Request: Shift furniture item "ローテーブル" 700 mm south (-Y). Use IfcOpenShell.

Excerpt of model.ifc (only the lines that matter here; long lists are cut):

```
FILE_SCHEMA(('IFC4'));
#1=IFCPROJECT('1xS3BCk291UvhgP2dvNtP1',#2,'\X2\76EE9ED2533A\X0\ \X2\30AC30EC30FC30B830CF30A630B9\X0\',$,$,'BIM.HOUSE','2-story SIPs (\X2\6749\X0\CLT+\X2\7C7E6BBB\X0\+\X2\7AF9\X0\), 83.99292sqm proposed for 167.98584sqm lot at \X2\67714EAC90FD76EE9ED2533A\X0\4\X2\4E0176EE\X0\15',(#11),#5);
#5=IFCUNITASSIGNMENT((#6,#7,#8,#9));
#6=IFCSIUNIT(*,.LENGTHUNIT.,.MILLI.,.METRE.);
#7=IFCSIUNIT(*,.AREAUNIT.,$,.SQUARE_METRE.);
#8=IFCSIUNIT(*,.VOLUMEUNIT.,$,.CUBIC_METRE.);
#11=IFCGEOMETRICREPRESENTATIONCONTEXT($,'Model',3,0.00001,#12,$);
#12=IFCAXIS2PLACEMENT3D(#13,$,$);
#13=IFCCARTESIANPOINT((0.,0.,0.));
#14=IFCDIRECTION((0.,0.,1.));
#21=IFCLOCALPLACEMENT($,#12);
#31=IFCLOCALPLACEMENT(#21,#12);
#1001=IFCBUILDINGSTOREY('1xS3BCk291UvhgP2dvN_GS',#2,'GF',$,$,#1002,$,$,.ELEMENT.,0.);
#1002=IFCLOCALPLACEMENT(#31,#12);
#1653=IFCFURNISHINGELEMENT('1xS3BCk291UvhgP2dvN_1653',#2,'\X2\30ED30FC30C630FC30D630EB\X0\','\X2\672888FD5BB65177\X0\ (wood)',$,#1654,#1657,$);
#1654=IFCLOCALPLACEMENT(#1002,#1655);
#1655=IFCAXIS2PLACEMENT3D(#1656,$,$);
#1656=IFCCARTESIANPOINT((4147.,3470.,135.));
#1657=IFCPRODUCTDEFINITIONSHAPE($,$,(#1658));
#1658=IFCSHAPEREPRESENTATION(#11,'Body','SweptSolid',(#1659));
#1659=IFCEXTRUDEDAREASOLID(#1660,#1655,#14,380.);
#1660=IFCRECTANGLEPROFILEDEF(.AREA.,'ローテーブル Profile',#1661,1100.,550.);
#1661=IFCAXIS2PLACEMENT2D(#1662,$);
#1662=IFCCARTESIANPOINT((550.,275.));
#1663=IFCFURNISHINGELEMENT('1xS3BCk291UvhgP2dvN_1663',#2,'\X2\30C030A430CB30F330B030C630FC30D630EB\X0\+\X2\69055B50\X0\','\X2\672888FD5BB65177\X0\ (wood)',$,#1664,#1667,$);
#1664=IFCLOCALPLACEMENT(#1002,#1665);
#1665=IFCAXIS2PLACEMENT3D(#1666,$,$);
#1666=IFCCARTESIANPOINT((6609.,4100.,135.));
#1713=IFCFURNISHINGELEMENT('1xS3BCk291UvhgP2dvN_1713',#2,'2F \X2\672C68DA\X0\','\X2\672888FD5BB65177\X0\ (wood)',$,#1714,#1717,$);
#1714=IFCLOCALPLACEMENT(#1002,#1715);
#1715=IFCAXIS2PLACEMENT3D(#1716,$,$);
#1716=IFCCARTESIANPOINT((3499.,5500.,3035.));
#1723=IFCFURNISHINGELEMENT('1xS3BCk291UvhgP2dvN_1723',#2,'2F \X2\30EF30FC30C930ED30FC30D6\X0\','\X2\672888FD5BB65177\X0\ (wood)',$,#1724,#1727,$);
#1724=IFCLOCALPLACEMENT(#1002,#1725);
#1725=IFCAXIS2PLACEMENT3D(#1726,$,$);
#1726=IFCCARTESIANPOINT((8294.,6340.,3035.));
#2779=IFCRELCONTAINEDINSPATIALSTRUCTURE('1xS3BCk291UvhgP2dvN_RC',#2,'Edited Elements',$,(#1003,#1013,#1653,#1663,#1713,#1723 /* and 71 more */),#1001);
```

```python
import ifcopenshell
import ifcopenshell.api.geometry
import ifcopenshell.util.placement
import ifcopenshell.util.unit

model = ifcopenshell.open("model.ifc")
unit_scale = ifcopenshell.util.unit.calculate_unit_scale(model)

item = model.by_guid("1xS3BCk291UvhgP2dvN_1653")
matrix = ifcopenshell.util.placement.get_local_placement(item.ObjectPlacement)
matrix[1, 3] -= 0.7 / unit_scale
ifcopenshell.api.geometry.edit_object_placement(model, product=item, matrix=matrix, is_si=False)

print(ifcopenshell.util.placement.get_local_placement(item.ObjectPlacement).round(3) + 0.0)

model.write("model_rev.ifc")
```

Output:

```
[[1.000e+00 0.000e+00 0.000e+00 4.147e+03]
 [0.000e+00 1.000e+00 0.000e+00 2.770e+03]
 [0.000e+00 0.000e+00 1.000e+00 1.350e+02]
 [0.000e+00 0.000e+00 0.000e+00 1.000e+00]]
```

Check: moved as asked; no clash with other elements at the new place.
